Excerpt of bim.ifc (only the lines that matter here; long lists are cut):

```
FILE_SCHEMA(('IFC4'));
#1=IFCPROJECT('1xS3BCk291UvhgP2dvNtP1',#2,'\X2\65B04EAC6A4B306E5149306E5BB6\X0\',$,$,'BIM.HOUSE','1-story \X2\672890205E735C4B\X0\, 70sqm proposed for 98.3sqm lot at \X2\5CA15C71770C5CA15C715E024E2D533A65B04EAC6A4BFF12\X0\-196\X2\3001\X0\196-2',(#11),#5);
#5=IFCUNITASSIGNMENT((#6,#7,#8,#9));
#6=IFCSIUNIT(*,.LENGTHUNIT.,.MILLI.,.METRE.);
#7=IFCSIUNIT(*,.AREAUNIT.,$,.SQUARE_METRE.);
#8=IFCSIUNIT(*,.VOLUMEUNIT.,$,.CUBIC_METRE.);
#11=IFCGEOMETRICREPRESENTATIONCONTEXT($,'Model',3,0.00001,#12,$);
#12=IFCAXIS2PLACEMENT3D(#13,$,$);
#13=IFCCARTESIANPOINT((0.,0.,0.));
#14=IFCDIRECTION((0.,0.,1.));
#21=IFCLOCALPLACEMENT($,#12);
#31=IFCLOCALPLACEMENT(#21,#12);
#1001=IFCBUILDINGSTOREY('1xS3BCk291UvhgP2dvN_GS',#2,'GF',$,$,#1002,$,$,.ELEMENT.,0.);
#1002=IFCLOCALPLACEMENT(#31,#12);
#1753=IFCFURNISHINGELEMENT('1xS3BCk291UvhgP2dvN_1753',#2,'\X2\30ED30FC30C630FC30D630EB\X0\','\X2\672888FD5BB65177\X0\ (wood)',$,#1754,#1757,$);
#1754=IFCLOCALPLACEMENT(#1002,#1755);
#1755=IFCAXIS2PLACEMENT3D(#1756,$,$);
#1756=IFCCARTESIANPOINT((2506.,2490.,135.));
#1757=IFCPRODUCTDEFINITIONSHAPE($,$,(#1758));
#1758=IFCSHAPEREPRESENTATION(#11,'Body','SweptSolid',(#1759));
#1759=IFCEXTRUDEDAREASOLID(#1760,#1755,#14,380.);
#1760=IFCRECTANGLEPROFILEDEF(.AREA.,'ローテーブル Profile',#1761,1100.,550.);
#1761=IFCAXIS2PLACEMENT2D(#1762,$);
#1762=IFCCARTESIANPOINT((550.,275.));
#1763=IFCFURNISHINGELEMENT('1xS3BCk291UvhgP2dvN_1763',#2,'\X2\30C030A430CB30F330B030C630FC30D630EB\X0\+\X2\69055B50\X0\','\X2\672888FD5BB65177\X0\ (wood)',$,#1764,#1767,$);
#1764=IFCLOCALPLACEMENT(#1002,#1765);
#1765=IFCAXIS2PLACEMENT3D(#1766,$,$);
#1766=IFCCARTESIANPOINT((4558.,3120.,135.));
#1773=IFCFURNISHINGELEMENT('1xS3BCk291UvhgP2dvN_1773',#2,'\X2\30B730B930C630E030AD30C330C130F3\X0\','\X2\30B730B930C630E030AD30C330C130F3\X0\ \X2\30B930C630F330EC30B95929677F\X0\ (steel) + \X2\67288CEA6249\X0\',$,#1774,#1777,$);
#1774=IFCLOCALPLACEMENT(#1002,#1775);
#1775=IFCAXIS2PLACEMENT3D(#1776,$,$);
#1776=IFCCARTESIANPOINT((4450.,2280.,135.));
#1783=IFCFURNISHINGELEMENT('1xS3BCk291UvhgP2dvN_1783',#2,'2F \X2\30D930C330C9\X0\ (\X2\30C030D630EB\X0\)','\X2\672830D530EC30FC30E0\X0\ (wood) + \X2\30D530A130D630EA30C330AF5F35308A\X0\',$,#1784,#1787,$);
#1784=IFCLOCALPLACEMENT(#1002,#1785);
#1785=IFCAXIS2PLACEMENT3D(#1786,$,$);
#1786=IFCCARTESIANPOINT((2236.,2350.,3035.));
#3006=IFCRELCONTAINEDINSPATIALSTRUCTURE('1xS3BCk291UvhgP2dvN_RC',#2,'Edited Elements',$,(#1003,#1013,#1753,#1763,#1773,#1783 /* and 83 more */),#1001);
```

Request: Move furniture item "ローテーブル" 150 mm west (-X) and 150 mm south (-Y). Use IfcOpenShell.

```python
import ifcopenshell
import ifcopenshell.api.geometry
import ifcopenshell.util.placement
import ifcopenshell.util.unit

model = ifcopenshell.open("bim.ifc")
unit_scale = ifcopenshell.util.unit.calculate_unit_scale(model)

item = model.by_guid("1xS3BCk291UvhgP2dvN_1753")
matrix = ifcopenshell.util.placement.get_local_placement(item.ObjectPlacement)
matrix[0, 3] -= 0.15 / unit_scale
matrix[1, 3] -= 0.15 / unit_scale
ifcopenshell.api.geometry.edit_object_placement(model, product=item, matrix=matrix, is_si=False)

print(ifcopenshell.util.placement.get_local_placement(item.ObjectPlacement).round(3) + 0.0)

model.write("bim_v2.ifc")
```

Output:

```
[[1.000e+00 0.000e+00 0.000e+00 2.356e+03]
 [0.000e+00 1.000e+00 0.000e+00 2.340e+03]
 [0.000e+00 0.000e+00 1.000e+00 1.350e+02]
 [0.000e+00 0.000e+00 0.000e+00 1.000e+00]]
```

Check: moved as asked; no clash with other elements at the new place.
